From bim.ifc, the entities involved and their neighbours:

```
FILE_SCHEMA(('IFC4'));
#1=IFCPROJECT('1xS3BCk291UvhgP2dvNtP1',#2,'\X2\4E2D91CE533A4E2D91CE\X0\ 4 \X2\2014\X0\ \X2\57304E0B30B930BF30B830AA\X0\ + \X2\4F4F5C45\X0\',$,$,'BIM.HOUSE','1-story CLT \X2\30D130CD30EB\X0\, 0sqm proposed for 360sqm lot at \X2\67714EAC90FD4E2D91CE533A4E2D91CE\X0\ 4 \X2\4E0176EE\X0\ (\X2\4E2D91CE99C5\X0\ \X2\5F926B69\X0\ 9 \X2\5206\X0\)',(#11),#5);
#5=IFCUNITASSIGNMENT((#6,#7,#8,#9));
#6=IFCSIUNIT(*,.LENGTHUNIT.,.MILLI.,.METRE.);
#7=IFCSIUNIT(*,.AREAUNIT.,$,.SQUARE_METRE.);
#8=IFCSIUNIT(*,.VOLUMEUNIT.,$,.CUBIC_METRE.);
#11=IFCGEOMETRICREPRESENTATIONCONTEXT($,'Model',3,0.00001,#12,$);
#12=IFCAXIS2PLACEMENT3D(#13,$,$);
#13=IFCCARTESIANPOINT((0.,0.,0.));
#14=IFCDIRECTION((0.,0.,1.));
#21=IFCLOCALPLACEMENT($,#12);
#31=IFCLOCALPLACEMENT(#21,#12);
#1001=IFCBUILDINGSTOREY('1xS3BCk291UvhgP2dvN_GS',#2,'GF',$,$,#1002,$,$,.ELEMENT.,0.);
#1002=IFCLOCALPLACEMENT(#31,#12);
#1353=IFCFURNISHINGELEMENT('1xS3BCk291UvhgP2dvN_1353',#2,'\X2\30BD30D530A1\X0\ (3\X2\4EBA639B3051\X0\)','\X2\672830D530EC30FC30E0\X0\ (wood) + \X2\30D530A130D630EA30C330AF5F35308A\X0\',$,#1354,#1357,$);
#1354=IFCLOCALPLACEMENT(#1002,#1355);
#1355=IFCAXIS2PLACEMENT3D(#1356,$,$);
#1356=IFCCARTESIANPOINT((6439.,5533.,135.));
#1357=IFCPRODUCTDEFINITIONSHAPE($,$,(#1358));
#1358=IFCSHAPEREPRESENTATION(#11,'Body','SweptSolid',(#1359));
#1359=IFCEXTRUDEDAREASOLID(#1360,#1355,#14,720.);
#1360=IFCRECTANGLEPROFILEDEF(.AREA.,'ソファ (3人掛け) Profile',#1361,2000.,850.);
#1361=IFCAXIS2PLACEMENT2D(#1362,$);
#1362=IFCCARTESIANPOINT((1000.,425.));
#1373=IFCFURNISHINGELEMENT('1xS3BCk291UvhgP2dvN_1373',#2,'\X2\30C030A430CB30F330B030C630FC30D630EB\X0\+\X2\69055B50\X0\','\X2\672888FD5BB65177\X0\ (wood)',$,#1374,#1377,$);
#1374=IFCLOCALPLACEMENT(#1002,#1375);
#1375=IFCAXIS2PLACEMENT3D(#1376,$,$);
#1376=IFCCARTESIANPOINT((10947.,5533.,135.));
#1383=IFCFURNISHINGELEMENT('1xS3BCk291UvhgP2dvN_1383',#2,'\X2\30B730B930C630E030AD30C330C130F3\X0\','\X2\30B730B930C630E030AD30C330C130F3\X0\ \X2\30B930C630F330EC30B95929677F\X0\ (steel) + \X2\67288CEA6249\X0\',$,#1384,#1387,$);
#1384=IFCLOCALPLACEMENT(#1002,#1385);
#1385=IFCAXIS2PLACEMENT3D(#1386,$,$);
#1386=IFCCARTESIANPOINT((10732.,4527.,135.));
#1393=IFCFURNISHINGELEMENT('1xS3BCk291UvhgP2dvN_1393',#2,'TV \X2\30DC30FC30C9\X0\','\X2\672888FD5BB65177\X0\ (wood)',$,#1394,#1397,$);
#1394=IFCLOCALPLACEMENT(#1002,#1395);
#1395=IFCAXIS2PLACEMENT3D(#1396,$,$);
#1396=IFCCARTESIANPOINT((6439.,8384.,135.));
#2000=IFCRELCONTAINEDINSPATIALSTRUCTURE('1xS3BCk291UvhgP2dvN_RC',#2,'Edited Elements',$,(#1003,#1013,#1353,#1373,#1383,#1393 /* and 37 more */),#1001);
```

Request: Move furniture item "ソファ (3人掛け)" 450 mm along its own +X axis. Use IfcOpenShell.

```python
import ifcopenshell
import ifcopenshell.api.geometry
import ifcopenshell.util.placement
import ifcopenshell.util.unit

model = ifcopenshell.open("bim.ifc")
unit_scale = ifcopenshell.util.unit.calculate_unit_scale(model)

item = model.by_guid("1xS3BCk291UvhgP2dvN_1353")
matrix = ifcopenshell.util.placement.get_local_placement(item.ObjectPlacement)
matrix[:3, 3] += matrix[:3, 0] * 0.45 / unit_scale
ifcopenshell.api.geometry.edit_object_placement(model, product=item, matrix=matrix, is_si=False)

print(ifcopenshell.util.placement.get_local_placement(item.ObjectPlacement).round(3) + 0.0)

model.write("bim-out.ifc")
```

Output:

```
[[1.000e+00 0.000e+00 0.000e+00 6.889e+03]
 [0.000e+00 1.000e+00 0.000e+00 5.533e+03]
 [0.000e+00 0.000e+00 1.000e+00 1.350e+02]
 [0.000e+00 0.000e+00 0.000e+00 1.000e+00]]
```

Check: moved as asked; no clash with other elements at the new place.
